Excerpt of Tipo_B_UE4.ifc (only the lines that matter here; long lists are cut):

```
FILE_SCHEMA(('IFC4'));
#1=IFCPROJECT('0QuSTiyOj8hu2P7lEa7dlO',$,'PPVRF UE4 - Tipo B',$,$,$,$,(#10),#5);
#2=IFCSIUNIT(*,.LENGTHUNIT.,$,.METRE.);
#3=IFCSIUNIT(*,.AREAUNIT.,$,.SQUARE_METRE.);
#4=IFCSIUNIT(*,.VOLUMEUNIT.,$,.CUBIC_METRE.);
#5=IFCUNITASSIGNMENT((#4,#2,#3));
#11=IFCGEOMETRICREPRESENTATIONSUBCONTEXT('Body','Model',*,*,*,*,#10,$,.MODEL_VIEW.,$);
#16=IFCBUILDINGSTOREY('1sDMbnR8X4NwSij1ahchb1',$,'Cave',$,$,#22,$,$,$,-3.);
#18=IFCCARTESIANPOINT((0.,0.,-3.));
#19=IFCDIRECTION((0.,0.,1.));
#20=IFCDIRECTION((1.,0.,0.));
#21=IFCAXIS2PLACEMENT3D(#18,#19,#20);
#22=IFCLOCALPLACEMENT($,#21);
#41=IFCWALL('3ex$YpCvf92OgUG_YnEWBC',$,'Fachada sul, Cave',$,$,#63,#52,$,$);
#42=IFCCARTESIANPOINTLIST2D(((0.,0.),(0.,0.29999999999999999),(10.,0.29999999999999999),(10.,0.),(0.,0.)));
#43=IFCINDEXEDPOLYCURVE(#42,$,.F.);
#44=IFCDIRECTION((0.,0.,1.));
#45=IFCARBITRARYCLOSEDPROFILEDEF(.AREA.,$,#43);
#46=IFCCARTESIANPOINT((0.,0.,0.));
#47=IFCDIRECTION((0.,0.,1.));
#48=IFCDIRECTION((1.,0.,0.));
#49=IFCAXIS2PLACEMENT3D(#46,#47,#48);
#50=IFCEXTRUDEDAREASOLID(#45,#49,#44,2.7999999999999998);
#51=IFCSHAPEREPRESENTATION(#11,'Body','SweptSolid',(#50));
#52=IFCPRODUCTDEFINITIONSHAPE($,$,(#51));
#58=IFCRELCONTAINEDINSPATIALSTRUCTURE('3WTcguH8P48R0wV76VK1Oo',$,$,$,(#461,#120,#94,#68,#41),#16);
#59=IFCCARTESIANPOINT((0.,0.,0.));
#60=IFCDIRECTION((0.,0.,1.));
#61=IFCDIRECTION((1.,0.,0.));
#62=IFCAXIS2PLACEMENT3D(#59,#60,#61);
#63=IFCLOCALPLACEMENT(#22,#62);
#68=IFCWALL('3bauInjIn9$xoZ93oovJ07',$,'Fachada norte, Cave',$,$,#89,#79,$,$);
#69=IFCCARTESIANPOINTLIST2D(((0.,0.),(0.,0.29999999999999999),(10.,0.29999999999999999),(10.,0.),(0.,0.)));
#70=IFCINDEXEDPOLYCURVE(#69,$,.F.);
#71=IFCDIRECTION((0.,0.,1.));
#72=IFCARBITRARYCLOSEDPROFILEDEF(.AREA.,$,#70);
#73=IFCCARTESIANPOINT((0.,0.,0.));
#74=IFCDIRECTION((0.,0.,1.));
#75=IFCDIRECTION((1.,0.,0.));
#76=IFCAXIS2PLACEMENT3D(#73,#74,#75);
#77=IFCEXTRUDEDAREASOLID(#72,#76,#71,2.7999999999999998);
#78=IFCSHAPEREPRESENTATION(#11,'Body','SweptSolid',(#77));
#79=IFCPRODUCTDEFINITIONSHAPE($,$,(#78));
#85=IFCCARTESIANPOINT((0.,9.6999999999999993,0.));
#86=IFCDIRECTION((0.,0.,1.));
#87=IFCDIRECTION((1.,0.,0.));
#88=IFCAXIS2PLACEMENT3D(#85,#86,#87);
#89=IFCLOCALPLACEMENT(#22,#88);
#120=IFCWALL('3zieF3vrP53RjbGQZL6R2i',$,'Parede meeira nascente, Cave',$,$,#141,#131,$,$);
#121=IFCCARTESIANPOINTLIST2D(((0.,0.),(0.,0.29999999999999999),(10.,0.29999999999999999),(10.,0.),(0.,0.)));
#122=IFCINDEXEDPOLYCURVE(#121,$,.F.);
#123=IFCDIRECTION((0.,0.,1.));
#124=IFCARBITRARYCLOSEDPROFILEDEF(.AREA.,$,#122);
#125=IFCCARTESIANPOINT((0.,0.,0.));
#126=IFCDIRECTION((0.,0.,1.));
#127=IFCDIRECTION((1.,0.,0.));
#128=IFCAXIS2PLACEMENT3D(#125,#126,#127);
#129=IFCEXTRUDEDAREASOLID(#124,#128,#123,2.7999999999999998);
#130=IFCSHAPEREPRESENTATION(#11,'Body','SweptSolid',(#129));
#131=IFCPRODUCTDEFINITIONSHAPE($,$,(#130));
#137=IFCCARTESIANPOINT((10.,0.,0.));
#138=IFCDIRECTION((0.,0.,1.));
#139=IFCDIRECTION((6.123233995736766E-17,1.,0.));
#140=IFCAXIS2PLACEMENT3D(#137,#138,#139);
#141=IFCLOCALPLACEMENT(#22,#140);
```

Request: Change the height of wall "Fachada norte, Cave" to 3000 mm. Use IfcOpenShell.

```python
import ifcopenshell
import ifcopenshell.geom
import ifcopenshell.util.representation
import ifcopenshell.util.shape
import ifcopenshell.util.unit

model = ifcopenshell.open("Tipo_B_UE4.ifc")
unit_scale = ifcopenshell.util.unit.calculate_unit_scale(model)
settings = ifcopenshell.geom.settings()


def volume(element):
    """Net volume in cubic metres, openings subtracted."""
    shape = ifcopenshell.geom.create_shape(settings, element)
    return ifcopenshell.util.shape.get_volume(shape.geometry)


wall = model.by_guid("3bauInjIn9$xoZ93oovJ07")
before = volume(wall)

body = ifcopenshell.util.representation.get_representation(wall, "Model", "Body")
solid = body.Items[0]
old_height = solid.Depth
solid.Depth = 3 / unit_scale
after = volume(wall)

print(f"height {old_height:g} -> {solid.Depth:g}, volume {before:.3f} -> {after:.3f} m3")

model.write("Tipo_B_UE4_updated.ifc")
```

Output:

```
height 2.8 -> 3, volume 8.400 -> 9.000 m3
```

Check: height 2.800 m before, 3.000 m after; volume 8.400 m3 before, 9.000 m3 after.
